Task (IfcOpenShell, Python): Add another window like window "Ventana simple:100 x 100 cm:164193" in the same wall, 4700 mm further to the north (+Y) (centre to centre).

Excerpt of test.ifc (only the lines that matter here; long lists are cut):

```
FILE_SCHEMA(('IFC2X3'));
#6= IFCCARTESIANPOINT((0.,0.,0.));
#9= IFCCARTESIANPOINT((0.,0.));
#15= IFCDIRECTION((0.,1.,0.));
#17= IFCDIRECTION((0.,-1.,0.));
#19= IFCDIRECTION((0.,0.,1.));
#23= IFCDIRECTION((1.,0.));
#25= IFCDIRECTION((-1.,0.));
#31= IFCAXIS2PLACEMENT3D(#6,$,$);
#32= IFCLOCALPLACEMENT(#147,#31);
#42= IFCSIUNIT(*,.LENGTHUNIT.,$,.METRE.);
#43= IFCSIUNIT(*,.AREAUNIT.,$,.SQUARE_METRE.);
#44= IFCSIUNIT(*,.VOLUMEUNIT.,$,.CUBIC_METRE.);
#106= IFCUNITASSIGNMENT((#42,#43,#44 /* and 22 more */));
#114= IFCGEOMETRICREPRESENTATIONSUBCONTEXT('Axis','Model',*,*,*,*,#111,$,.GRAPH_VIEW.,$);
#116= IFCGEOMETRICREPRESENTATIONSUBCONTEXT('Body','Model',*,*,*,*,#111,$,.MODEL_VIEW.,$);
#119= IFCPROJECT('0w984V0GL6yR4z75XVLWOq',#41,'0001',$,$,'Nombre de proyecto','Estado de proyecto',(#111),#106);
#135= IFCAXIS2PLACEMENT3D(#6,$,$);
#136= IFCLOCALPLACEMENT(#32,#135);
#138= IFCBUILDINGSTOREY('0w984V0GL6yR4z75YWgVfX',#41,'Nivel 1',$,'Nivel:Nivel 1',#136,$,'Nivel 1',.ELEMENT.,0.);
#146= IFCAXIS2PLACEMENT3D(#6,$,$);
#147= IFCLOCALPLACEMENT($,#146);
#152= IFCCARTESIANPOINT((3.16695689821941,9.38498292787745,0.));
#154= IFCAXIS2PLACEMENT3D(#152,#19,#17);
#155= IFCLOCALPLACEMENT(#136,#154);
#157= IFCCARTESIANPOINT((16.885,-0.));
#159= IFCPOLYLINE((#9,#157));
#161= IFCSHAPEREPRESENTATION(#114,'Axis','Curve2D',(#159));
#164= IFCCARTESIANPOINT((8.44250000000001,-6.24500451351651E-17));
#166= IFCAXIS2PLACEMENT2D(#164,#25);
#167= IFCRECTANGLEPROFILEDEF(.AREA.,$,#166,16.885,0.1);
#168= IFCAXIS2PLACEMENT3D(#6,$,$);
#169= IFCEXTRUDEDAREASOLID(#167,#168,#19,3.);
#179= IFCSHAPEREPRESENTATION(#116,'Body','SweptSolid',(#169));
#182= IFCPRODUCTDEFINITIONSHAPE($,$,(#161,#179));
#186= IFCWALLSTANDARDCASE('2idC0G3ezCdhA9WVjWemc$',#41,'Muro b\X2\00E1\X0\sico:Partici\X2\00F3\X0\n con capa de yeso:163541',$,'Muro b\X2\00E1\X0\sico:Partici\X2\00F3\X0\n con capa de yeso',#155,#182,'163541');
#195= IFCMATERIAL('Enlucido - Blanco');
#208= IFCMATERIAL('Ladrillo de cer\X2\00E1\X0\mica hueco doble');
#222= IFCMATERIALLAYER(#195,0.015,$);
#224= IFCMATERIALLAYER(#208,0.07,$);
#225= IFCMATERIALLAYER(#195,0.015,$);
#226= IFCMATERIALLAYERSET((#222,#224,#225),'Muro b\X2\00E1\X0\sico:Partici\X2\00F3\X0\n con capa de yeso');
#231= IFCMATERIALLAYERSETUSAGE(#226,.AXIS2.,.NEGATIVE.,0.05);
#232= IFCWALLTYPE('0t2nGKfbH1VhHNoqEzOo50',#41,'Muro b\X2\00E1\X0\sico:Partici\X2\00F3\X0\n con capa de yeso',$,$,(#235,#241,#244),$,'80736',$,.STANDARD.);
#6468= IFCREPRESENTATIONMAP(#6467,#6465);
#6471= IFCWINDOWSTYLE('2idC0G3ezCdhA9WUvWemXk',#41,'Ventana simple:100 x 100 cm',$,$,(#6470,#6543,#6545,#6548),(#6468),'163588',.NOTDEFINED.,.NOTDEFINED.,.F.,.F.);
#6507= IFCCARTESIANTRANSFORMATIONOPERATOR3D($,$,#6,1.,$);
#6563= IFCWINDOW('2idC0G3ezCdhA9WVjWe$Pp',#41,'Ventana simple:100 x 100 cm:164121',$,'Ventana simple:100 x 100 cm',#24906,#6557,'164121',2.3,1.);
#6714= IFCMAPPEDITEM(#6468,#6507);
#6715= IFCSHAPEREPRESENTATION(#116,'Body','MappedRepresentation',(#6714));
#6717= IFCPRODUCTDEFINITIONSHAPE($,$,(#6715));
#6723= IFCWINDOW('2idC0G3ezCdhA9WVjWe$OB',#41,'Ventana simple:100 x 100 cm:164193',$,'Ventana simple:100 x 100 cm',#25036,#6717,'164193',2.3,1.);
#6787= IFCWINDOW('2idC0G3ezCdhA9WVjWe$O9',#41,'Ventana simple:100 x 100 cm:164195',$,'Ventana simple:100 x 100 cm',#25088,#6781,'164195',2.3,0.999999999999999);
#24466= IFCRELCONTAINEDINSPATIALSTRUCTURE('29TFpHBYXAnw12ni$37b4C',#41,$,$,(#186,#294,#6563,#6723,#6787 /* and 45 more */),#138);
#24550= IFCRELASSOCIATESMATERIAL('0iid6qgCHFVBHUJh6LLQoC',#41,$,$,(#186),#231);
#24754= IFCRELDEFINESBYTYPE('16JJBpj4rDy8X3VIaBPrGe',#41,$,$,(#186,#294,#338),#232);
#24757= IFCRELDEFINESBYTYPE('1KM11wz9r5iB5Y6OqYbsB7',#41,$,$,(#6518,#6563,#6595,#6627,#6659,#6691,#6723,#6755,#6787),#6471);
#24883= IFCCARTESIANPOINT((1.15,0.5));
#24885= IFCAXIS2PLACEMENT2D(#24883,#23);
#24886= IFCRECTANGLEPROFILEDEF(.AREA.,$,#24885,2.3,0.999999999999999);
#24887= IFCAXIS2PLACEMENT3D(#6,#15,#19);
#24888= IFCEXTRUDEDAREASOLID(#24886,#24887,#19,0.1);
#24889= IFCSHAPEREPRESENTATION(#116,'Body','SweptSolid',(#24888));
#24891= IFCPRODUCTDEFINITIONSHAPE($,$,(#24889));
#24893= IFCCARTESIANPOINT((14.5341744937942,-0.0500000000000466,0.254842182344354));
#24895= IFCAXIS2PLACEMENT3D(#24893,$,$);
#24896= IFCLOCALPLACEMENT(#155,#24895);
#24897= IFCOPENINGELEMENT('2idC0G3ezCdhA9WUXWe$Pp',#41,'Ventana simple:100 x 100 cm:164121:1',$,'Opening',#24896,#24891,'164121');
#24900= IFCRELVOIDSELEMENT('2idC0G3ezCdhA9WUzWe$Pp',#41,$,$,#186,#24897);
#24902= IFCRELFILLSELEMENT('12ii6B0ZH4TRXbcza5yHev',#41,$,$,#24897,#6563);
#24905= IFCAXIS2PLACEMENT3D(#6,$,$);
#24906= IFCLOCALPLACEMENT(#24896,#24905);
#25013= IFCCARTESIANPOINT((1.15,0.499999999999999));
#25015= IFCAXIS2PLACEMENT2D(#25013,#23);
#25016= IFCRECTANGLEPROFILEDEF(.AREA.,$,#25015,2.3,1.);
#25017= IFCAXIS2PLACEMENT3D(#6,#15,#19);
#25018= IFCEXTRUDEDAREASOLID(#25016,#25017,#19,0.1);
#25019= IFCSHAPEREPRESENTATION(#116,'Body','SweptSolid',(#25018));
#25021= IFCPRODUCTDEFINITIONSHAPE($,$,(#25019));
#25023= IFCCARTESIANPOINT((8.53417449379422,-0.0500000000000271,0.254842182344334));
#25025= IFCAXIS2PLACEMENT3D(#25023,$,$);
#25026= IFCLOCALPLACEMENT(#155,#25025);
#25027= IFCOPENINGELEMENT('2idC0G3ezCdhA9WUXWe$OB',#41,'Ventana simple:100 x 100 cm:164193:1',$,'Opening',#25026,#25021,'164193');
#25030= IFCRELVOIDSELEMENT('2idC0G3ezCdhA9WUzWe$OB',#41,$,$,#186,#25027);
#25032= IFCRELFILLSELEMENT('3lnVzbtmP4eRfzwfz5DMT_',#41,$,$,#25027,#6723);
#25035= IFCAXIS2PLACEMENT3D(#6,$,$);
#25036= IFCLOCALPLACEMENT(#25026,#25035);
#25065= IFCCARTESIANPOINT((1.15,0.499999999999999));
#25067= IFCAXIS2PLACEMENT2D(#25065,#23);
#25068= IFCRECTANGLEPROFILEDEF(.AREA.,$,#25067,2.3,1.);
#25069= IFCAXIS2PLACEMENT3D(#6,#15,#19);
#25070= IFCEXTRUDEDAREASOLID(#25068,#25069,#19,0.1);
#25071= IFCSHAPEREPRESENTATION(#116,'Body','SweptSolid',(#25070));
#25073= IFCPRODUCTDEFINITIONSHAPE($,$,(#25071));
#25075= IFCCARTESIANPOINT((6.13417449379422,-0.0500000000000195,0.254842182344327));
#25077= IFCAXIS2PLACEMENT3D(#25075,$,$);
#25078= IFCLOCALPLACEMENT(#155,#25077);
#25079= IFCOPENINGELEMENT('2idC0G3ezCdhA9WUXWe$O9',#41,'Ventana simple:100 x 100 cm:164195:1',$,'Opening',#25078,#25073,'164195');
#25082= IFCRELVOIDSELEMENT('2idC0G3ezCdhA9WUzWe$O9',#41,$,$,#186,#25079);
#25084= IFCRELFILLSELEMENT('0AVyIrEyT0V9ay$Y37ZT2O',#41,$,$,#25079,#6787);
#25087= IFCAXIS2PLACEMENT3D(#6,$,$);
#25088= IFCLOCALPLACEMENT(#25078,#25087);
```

```python
import ifcopenshell
import ifcopenshell.api.feature
import ifcopenshell.api.geometry
import ifcopenshell.api.root
import ifcopenshell.geom
import ifcopenshell.util.element
import ifcopenshell.util.placement
import ifcopenshell.util.shape

model = ifcopenshell.open("test.ifc")
settings = ifcopenshell.geom.settings()


def volume(element):
    """Net volume in cubic metres, openings subtracted."""
    shape = ifcopenshell.geom.create_shape(settings, element)
    return ifcopenshell.util.shape.get_volume(shape.geometry)


def reuse_history(source, copy):
    """copy_class also copies each property set's owner history, people and application; keep the originals."""
    for rel in copy.IsDefinedBy:
        if rel.is_a("IfcRelDefinesByProperties") and (history := rel.RelatingPropertyDefinition.OwnerHistory):
            rel.RelatingPropertyDefinition.OwnerHistory = source.OwnerHistory
            ifcopenshell.util.element.remove_deep2(model, history)


window = model.by_guid("2idC0G3ezCdhA9WVjWe$OB")
opening = window.FillsVoids[0].RelatingOpeningElement
wall = opening.VoidsElements[0].RelatingBuildingElement
before = volume(wall)
shift = ifcopenshell.util.placement.get_local_placement(wall.ObjectPlacement)[:3, 0] * -4.7

# copy_class copies the void relationship, type, container and properties, but no geometry.
new_opening = ifcopenshell.api.root.copy_class(model, product=opening)
new_opening.Representation = ifcopenshell.util.element.copy_deep(
    model, opening.Representation, exclude=["IfcGeometricRepresentationContext", "IfcRepresentationMap"]
)
new_opening.Name = "Ventana simple:100 x 100 cm"
new_opening.Tag = None
new_window = ifcopenshell.api.root.copy_class(model, product=window)
new_window.Representation = ifcopenshell.util.element.copy_deep(
    model, window.Representation, exclude=["IfcGeometricRepresentationContext", "IfcRepresentationMap"]
)
new_window.Name = "Ventana simple:100 x 100 cm"
new_window.Tag = None
reuse_history(window, new_window)
fills = ifcopenshell.api.feature.add_filling(model, opening=new_opening, element=new_window)
fills.OwnerHistory = new_window.OwnerHistory  # required in IFC2X3

for old, new in ((opening, new_opening), (window, new_window)):
    matrix = ifcopenshell.util.placement.get_local_placement(old.ObjectPlacement)
    matrix[:3, 3] += shift
    ifcopenshell.api.geometry.edit_object_placement(model, product=new, matrix=matrix, is_si=False)

after = volume(wall)

print(f"wall volume {before:.3f} -> {after:.3f} m3")

model.write("test_updated.ifc")
```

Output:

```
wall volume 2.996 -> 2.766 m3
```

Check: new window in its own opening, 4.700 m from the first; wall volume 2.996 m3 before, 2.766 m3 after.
